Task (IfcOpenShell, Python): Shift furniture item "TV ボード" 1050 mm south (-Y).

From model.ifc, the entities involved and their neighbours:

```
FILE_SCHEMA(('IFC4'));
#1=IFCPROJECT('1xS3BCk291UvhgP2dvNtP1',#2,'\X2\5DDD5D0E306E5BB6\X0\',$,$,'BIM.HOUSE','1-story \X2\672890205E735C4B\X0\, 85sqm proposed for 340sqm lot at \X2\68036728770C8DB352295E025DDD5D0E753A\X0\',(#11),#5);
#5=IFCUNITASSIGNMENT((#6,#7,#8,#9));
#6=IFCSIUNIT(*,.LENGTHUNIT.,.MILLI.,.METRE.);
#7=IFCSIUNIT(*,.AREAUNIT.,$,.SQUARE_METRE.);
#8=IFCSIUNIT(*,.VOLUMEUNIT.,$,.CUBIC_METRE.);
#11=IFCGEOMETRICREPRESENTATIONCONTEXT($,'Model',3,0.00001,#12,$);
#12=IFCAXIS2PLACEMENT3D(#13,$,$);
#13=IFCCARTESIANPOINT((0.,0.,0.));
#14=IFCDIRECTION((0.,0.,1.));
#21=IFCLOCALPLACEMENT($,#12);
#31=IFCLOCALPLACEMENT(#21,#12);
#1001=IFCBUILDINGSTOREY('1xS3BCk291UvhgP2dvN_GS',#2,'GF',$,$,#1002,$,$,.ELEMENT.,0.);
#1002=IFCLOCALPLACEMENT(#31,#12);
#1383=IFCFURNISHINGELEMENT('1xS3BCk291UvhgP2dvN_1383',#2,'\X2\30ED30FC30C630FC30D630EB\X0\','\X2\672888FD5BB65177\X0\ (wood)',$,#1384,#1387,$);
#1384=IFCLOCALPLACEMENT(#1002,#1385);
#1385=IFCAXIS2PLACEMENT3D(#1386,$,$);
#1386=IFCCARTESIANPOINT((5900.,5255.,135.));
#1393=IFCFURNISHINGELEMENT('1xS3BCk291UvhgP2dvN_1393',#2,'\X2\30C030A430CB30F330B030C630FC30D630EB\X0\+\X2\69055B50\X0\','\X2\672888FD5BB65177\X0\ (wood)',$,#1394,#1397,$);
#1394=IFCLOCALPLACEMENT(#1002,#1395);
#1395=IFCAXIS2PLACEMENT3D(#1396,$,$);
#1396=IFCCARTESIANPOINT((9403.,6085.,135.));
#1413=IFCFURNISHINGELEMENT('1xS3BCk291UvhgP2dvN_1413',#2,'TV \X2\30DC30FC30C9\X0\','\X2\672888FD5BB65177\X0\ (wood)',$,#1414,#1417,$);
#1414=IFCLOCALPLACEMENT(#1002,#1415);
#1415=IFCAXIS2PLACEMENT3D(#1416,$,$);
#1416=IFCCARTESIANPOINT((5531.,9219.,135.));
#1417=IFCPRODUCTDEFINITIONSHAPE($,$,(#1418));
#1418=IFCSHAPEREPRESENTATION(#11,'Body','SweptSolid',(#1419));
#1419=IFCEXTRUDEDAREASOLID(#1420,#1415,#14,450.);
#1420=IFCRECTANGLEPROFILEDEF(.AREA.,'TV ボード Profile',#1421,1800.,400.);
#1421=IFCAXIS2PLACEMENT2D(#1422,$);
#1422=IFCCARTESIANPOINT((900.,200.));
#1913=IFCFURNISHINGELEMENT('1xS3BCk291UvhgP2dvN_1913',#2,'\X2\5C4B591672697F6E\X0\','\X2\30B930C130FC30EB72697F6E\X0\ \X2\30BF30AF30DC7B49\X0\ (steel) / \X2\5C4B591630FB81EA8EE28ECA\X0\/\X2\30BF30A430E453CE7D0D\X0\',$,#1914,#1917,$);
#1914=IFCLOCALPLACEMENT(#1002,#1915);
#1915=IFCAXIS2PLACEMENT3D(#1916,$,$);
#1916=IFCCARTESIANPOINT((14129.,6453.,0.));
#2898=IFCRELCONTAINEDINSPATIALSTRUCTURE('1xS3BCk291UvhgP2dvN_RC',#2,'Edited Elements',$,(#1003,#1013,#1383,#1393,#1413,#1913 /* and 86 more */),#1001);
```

```python
import ifcopenshell
import ifcopenshell.api.geometry
import ifcopenshell.util.placement

model = ifcopenshell.open("model.ifc")

item = model.by_guid("1xS3BCk291UvhgP2dvN_1413")
matrix = ifcopenshell.util.placement.get_local_placement(item.ObjectPlacement)
matrix[1, 3] -= 1050.0
ifcopenshell.api.geometry.edit_object_placement(model, product=item, matrix=matrix, is_si=False)

print(ifcopenshell.util.placement.get_local_placement(item.ObjectPlacement).round(3) + 0.0)

model.write("model_updated.ifc")
```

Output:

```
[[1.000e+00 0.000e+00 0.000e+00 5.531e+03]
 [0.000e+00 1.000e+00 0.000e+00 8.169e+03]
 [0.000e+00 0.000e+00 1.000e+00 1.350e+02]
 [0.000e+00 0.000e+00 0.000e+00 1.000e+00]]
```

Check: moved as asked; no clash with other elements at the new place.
